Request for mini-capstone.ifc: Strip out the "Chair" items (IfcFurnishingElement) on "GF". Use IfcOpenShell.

First a look at what the model holds.

```python
import ifcopenshell
import ifcopenshell.util.element

model = ifcopenshell.open("mini-capstone.ifc")
print(model.schema)
storey = next(s for s in model.by_type("IfcBuildingStorey") if s.Name == "GF")
furniture = [e for e in ifcopenshell.util.element.get_decomposition(storey) if e.is_a("IfcFurnishingElement")]
seen = {}
for e in furniture:
    element_type = ifcopenshell.util.element.get_type(e)
    name = element_type.Name if element_type not in (None, e) else None
    seen[name] = seen.get(name, 0) + 1
for name, count in sorted(seen.items(), key=str):
    print(count, "x", name)
```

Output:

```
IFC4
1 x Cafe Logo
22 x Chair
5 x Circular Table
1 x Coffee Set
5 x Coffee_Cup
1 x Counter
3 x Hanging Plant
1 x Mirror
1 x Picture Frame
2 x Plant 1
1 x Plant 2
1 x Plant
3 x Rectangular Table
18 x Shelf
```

```python
import ifcopenshell
import ifcopenshell.api.root
import ifcopenshell.util.element

model = ifcopenshell.open("mini-capstone.ifc")

storey = next(s for s in model.by_type("IfcBuildingStorey") if s.Name == "GF")
furniture = [e for e in ifcopenshell.util.element.get_decomposition(storey) if e.is_a("IfcFurnishingElement")]
targets = [e for e in furniture if (t := ifcopenshell.util.element.get_type(e)) not in (None, e) and t.Name == "Chair"]

for e in targets:
    ifcopenshell.api.root.remove_product(model, product=e)
print(len(targets), "removed")

model.write("mini-capstone_edited.ifc")
```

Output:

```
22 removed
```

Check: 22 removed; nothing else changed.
